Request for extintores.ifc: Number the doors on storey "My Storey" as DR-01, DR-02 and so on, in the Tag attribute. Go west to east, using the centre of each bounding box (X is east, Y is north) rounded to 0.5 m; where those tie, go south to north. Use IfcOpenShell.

First a look at what the model holds.

```python
import ifcopenshell
import ifcopenshell.util.element
import ifcopenshell.util.placement

model = ifcopenshell.open("extintores.ifc")
print(model.schema)
storey = next(s for s in model.by_type("IfcBuildingStorey") if s.Name == "My Storey")
doors = [e for e in ifcopenshell.util.element.get_decomposition(storey) if e.is_a("IfcDoor")]
for e in sorted(doors, key=lambda e: e.id()):
    origin = ifcopenshell.util.placement.get_local_placement(e.ObjectPlacement)[:3, 3]
    print(e.id(), e.Tag, e.Name, origin.round(2) + 0.0, sep=" | ")
```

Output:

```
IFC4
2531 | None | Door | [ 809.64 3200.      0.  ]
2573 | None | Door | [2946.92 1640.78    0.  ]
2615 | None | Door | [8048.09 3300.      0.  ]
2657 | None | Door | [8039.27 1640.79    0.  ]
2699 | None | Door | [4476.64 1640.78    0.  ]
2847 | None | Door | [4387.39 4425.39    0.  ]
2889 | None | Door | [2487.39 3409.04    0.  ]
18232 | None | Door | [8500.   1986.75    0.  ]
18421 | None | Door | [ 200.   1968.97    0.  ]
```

```python
import ifcopenshell
import ifcopenshell.geom
import ifcopenshell.util.element
import ifcopenshell.util.shape

model = ifcopenshell.open("extintores.ifc")
settings = ifcopenshell.geom.settings()
settings.set("use-world-coords", True)


def centre(element):
    shape = ifcopenshell.geom.create_shape(settings, element)
    return ifcopenshell.util.shape.get_bbox_centroid(shape.geometry)


storey = next(s for s in model.by_type("IfcBuildingStorey") if s.Name == "My Storey")
doors = [e for e in ifcopenshell.util.element.get_decomposition(storey) if e.is_a("IfcDoor")]

# Insertion points can sit at a corner or the storey origin, so sort by the geometry (in metres).
centres = {e: centre(e) for e in doors}
doors.sort(key=lambda e: (round(centres[e][0] / 0.5), centres[e][1]))

for i, e in enumerate(doors, start=1):
    number = f"DR-{i:02d}"
    e.Tag = number
    print(e.id(), number)

model.write("extintores_v2.ifc")
```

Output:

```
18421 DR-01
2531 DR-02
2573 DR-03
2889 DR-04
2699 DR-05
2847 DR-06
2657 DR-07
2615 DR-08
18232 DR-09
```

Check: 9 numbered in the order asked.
